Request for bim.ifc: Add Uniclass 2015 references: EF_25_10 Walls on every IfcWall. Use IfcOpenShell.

First a look at what the model holds.

```python
import ifcopenshell

model = ifcopenshell.open("bim.ifc")
print(model.schema)
print("classifications:", [c.Name for c in model.by_type("IfcClassification")])
for ifc_class in ("IfcDoor", "IfcRoof", "IfcStair", "IfcWall", "IfcWindow"):
    print(ifc_class, len(model.by_type(ifc_class)))
```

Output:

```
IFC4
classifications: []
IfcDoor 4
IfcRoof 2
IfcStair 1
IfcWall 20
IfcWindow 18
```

```python
import ifcopenshell
import ifcopenshell.api.classification

model = ifcopenshell.open("bim.ifc")

system = ifcopenshell.api.classification.add_classification(model, classification="Uniclass 2015")

codes = {
    "IfcWall": ("EF_25_10", "Walls"),
}
for ifc_class, (code, name) in codes.items():
    products = model.by_type(ifc_class)
    ifcopenshell.api.classification.add_reference(
        model, products=products, classification=system, identification=code, name=name
    )
    print(code, len(products))

model.write("bim_v2.ifc")
```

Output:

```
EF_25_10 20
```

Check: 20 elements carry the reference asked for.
